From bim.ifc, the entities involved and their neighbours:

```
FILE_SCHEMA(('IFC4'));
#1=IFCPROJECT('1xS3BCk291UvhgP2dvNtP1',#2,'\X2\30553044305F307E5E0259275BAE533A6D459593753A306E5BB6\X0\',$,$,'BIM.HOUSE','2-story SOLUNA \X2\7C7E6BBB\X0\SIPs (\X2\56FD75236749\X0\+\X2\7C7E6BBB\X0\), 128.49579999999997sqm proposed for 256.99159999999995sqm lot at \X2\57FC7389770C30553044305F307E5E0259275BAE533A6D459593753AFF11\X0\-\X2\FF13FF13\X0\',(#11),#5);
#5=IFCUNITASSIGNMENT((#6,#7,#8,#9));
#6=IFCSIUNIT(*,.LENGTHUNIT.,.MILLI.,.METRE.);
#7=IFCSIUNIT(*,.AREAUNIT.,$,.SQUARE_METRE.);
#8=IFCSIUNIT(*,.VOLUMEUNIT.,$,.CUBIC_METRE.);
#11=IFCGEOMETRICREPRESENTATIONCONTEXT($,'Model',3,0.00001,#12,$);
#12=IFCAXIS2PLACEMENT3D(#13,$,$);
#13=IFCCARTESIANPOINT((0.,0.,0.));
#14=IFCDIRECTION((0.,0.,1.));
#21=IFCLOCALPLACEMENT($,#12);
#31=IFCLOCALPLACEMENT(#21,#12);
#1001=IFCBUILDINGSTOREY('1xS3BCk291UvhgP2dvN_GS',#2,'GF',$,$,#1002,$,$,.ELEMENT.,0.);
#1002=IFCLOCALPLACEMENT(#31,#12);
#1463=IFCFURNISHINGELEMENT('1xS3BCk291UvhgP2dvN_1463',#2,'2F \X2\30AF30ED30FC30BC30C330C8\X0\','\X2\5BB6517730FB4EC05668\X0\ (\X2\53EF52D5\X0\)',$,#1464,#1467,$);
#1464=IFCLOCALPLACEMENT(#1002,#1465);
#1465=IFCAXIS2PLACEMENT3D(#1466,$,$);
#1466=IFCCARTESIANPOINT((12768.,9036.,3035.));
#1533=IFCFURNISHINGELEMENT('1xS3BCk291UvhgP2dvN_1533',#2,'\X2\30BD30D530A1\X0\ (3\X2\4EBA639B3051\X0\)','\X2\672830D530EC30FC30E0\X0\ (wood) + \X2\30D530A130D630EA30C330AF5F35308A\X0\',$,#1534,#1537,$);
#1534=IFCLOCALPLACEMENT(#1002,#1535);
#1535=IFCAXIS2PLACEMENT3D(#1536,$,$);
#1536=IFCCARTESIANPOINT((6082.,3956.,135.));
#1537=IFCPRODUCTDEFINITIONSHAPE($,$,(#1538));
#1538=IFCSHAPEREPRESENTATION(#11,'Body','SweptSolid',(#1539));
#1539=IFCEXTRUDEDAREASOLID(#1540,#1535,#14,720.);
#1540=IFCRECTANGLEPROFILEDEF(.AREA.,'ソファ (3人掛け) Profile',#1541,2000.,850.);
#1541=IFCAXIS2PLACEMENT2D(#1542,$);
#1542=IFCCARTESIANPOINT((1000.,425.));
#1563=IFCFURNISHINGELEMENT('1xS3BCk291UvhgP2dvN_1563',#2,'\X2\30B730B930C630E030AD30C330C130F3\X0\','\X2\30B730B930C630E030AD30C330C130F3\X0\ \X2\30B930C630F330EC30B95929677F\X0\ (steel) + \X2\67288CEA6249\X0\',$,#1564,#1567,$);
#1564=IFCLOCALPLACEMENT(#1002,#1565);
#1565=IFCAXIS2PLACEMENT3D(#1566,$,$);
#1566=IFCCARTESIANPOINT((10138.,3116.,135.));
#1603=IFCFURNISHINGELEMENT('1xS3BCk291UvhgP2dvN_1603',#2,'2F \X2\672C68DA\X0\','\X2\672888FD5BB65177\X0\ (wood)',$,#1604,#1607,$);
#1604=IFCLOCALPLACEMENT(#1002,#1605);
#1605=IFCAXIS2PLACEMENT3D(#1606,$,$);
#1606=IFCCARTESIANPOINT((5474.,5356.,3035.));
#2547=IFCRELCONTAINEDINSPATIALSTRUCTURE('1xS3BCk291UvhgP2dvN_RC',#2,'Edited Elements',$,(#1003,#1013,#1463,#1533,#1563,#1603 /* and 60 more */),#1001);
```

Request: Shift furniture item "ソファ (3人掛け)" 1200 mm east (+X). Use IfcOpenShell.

```python
import ifcopenshell
import ifcopenshell.api.geometry
import ifcopenshell.util.placement
import ifcopenshell.util.unit

model = ifcopenshell.open("bim.ifc")
unit_scale = ifcopenshell.util.unit.calculate_unit_scale(model)

item = model.by_id(1533)
matrix = ifcopenshell.util.placement.get_local_placement(item.ObjectPlacement)
matrix[0, 3] += 1.2 / unit_scale
ifcopenshell.api.geometry.edit_object_placement(model, product=item, matrix=matrix, is_si=False)

print(ifcopenshell.util.placement.get_local_placement(item.ObjectPlacement).round(3) + 0.0)

model.write("bim-out.ifc")
```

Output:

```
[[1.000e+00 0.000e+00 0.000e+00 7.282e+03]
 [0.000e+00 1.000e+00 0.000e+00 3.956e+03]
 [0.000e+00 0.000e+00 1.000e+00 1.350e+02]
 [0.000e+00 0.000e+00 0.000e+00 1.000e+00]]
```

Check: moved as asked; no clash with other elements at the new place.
